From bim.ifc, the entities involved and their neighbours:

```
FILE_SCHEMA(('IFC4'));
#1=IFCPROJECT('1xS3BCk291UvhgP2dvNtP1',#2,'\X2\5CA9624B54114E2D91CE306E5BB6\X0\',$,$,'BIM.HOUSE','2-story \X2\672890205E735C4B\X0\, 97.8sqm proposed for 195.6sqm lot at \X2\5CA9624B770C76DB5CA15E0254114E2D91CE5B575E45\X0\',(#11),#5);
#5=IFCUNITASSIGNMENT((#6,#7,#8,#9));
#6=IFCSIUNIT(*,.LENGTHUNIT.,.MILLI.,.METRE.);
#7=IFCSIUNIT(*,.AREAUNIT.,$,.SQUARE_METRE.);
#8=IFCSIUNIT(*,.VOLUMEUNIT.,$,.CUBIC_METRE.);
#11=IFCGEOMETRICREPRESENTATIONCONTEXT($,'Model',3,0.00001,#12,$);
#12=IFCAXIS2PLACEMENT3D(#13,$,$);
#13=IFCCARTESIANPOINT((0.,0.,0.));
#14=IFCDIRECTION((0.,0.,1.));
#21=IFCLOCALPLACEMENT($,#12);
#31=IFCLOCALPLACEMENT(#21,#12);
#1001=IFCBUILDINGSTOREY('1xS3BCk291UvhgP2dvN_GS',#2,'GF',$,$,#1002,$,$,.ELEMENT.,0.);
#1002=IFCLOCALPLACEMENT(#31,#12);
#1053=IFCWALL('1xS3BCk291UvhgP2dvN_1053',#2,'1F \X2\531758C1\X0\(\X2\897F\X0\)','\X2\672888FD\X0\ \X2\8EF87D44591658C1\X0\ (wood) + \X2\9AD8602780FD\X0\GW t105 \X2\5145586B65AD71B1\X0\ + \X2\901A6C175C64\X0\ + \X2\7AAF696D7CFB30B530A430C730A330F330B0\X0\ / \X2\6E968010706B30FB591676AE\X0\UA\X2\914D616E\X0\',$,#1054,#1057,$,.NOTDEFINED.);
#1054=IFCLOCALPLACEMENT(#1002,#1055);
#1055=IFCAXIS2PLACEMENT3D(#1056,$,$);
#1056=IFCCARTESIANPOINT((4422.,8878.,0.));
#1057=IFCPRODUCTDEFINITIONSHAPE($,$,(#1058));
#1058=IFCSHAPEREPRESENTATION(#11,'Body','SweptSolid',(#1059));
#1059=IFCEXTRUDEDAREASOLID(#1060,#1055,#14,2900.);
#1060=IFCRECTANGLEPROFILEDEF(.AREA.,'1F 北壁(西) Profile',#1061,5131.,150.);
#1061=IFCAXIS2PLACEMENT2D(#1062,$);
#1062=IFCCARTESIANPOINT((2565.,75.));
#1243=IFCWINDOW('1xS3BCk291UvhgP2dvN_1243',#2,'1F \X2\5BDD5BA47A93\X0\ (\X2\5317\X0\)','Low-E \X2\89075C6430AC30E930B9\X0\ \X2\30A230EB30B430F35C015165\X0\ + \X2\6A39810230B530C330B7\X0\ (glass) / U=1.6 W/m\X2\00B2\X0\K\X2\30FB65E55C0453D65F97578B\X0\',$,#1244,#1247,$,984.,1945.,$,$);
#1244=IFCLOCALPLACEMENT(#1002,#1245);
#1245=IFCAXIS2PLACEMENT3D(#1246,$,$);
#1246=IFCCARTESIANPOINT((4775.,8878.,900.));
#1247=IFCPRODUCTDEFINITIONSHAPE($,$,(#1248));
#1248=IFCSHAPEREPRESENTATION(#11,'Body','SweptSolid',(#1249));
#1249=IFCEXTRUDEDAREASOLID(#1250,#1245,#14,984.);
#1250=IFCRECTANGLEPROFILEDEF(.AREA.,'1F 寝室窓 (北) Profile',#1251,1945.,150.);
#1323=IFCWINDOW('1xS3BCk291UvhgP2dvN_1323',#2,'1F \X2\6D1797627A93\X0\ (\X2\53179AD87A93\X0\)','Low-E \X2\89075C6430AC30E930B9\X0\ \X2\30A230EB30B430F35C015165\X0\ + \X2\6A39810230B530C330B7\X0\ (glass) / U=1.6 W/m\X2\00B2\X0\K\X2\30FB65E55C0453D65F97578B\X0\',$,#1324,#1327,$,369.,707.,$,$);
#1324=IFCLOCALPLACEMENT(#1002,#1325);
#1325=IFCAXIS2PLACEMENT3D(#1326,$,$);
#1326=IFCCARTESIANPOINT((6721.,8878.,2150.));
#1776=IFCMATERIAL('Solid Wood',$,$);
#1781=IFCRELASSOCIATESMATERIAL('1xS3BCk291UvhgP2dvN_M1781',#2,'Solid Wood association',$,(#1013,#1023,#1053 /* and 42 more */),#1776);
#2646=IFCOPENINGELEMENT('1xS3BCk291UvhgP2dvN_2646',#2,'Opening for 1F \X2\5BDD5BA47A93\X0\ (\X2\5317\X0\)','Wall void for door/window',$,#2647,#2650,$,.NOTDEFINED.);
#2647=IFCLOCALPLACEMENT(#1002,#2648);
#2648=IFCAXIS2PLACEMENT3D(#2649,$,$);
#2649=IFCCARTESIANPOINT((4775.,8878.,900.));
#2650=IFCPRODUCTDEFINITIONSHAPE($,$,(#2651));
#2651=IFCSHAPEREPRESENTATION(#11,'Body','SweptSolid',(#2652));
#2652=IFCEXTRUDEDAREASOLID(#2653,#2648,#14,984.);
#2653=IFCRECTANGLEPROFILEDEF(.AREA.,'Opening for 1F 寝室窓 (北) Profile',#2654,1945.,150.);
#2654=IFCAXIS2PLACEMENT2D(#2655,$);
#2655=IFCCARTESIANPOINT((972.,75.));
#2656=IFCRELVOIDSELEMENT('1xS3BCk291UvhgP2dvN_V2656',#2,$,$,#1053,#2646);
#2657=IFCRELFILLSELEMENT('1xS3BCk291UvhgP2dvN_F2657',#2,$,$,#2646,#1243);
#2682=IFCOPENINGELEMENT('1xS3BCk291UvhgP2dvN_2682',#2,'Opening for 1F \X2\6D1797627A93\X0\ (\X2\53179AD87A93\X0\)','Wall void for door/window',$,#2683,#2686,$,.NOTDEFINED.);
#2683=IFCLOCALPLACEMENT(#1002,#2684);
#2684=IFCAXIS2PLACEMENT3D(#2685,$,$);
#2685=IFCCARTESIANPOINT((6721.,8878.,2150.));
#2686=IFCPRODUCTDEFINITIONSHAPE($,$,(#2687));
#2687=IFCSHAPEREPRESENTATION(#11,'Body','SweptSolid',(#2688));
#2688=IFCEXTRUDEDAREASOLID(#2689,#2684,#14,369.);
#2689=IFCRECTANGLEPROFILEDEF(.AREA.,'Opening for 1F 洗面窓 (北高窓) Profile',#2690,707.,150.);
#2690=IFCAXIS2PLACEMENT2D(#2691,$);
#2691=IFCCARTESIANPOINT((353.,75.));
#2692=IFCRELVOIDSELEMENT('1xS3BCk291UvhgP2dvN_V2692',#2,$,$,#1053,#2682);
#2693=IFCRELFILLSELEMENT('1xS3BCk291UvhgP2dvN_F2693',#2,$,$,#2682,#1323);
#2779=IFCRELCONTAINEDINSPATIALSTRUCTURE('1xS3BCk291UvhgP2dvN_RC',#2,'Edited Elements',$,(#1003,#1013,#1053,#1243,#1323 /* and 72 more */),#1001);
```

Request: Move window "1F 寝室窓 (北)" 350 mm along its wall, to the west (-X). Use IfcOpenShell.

```python
import ifcopenshell
import ifcopenshell.api.geometry
import ifcopenshell.util.placement

model = ifcopenshell.open("bim.ifc")

window = model.by_guid("1xS3BCk291UvhgP2dvN_1243")
opening = window.FillsVoids[0].RelatingOpeningElement
wall = opening.VoidsElements[0].RelatingBuildingElement

wall_matrix = ifcopenshell.util.placement.get_local_placement(wall.ObjectPlacement)
shift = wall_matrix[:3, 0] * -350.0
before = ifcopenshell.util.placement.get_local_placement(window.ObjectPlacement)[:3, 3].copy()

# The window is not placed relative to its opening, so move both.
for product in (opening, window):
    matrix = ifcopenshell.util.placement.get_local_placement(product.ObjectPlacement)
    matrix[:3, 3] += shift
    ifcopenshell.api.geometry.edit_object_placement(model, product=product, matrix=matrix, is_si=False)

after = ifcopenshell.util.placement.get_local_placement(window.ObjectPlacement)[:3, 3]
print("window moved by", (after - before).round(3) + 0.0)

model.write("bim-out.ifc")
```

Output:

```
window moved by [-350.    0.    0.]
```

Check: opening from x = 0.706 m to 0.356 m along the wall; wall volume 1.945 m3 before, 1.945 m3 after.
